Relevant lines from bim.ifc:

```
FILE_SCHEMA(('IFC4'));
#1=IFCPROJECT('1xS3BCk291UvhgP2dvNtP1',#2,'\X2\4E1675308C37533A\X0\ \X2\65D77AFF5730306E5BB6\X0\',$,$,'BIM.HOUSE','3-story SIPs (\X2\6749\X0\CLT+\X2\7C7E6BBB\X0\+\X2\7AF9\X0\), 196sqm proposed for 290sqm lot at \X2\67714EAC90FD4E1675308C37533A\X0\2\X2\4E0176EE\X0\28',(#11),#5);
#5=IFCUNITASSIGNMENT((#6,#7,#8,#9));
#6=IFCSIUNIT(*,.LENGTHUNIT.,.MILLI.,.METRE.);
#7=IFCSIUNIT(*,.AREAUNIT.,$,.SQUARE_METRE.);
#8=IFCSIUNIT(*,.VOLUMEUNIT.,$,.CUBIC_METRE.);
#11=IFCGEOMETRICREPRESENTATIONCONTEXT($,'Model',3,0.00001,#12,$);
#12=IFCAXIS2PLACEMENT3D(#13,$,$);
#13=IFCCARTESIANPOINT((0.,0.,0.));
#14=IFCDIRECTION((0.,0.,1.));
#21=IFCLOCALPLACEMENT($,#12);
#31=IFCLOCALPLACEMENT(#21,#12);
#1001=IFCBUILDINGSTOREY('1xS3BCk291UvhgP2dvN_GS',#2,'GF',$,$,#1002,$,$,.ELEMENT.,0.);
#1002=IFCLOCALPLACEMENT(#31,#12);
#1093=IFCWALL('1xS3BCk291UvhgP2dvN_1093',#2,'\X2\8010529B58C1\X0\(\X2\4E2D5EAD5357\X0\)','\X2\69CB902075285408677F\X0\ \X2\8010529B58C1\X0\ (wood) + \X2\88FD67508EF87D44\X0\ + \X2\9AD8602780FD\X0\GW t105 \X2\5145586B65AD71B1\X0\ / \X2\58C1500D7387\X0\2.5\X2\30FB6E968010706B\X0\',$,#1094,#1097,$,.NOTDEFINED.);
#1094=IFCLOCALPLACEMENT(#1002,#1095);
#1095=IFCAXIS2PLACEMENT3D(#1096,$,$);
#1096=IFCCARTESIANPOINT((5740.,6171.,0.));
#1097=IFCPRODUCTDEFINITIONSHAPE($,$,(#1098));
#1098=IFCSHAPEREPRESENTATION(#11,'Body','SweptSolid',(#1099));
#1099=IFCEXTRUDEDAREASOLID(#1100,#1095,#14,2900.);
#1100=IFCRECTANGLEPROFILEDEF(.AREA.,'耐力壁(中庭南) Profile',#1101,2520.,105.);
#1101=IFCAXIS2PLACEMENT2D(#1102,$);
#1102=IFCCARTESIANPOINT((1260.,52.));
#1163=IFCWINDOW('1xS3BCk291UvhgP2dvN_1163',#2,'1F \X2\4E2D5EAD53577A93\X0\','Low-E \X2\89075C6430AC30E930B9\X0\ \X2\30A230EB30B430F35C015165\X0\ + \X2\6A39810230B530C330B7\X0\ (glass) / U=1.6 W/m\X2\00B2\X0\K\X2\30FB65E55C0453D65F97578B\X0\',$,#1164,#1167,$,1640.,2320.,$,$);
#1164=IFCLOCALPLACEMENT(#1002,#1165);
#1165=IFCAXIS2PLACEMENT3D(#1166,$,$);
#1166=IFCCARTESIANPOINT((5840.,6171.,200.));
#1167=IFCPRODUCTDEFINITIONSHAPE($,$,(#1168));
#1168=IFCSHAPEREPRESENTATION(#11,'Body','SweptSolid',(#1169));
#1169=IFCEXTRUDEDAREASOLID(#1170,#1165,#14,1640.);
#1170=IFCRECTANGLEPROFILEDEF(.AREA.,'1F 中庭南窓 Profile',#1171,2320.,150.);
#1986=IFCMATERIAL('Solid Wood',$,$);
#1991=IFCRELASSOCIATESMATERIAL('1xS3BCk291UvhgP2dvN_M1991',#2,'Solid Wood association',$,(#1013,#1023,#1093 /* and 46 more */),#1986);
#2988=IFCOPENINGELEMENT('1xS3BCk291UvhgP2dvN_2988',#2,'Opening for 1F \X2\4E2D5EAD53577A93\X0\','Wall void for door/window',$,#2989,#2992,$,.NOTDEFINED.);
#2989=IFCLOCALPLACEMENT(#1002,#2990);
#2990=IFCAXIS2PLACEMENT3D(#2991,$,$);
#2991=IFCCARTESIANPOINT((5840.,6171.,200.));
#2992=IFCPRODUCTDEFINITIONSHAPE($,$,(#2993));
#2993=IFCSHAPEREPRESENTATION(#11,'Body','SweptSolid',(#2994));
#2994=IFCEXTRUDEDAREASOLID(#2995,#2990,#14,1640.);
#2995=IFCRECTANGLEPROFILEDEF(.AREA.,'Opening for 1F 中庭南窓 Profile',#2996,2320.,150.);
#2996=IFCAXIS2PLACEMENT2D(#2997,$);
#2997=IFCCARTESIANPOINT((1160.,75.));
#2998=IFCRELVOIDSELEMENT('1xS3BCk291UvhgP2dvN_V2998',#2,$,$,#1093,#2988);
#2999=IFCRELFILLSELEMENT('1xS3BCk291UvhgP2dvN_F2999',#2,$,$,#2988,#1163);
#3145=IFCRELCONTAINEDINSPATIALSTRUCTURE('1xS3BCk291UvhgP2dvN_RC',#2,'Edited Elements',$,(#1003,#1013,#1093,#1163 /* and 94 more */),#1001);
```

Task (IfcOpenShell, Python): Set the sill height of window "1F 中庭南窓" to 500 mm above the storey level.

```python
import numpy as np
import ifcopenshell
import ifcopenshell.api.geometry
import ifcopenshell.geom
import ifcopenshell.util.element
import ifcopenshell.util.placement
import ifcopenshell.util.shape
import ifcopenshell.util.unit

model = ifcopenshell.open("bim.ifc")
unit_scale = ifcopenshell.util.unit.calculate_unit_scale(model)

window = model.by_guid("1xS3BCk291UvhgP2dvN_1163")
opening = window.FillsVoids[0].RelatingOpeningElement
storey = ifcopenshell.util.element.get_container(window, ifc_class="IfcBuildingStorey")
level = ifcopenshell.util.placement.get_local_placement(storey.ObjectPlacement)[2, 3]

# The opening's origin need not be at the sill, so measure its lowest point.
shape = ifcopenshell.geom.create_shape(ifcopenshell.geom.settings(), opening)
bottom = ifcopenshell.util.shape.get_shape_bottom_elevation(shape, shape.geometry) / unit_scale
dz = level + 0.5 / unit_scale - bottom

shift = np.array([0.0, 0.0, dz])
# The window is not placed relative to its opening, so move both.
for product in (opening, window):
    matrix = ifcopenshell.util.placement.get_local_placement(product.ObjectPlacement)
    matrix[:3, 3] += shift
    ifcopenshell.api.geometry.edit_object_placement(model, product=product, matrix=matrix, is_si=False)

print(f"moved by {dz * unit_scale:+.3f} m")

model.write("bim_v2.ifc")
```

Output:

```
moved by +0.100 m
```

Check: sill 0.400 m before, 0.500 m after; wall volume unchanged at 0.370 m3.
